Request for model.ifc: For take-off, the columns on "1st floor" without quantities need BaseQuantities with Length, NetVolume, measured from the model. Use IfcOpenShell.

First a look at what the model holds.

```python
import ifcopenshell
import ifcopenshell.util.element
import ifcopenshell.util.unit

model = ifcopenshell.open("model.ifc")
print(model.schema)
for unit_type in ("LENGTHUNIT", "AREAUNIT", "VOLUMEUNIT"):
    print(unit_type, ifcopenshell.util.unit.calculate_unit_scale(model, unit_type))
storey = next(s for s in model.by_type("IfcBuildingStorey") if s.Name == "1st floor")
columns = [e for e in ifcopenshell.util.element.get_decomposition(storey) if e.is_a("IfcColumn")]
for e in sorted(columns, key=lambda e: e.id()):
    print(e.id(), e.is_a(), e.Name, list(ifcopenshell.util.element.get_psets(e, qtos_only=True)), sep=" | ")
```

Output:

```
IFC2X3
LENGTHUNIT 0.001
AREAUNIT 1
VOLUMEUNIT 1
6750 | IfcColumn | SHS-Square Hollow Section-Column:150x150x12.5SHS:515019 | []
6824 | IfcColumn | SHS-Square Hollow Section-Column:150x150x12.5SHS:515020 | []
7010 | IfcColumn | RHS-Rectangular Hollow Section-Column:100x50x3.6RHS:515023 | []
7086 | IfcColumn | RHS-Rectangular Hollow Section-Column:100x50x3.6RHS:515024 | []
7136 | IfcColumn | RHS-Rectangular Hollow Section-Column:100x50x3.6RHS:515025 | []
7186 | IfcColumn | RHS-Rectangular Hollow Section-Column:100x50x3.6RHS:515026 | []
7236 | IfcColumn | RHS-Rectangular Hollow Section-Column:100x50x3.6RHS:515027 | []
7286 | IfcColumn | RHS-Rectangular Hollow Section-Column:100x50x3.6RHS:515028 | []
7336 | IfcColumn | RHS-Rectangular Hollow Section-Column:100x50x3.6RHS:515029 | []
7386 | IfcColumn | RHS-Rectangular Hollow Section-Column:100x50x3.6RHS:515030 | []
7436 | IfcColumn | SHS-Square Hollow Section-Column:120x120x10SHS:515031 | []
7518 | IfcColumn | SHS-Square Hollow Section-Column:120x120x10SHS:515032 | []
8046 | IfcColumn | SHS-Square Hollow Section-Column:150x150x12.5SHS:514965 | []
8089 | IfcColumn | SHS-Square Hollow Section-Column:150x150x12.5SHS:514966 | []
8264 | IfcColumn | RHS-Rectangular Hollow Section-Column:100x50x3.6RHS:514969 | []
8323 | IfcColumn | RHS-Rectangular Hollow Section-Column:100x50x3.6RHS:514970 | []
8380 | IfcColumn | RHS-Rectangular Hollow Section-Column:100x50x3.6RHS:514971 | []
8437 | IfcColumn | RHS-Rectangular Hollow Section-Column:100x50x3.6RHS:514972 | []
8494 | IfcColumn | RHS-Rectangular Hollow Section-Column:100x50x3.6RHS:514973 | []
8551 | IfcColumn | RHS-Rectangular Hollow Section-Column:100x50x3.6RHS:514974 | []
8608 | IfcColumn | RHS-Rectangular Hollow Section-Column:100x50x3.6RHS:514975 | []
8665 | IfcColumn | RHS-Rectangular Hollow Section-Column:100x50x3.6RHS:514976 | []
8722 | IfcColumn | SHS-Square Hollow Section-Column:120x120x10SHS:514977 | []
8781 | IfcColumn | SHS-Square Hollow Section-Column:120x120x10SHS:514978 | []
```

```python
import ifcopenshell
import ifcopenshell.api.pset
import ifcopenshell.geom
import ifcopenshell.util.element
import ifcopenshell.util.shape
import ifcopenshell.util.unit

model = ifcopenshell.open("model.ifc")
unit_scale = ifcopenshell.util.unit.calculate_unit_scale(model)
volume_scale = ifcopenshell.util.unit.calculate_unit_scale(model, "VOLUMEUNIT")
settings = ifcopenshell.geom.settings()

storey = next(s for s in model.by_type("IfcBuildingStorey") if s.Name == "1st floor")
columns = [e for e in ifcopenshell.util.element.get_decomposition(storey) if e.is_a("IfcColumn")]

for e in sorted(columns, key=lambda e: e.id()):
    if ifcopenshell.util.element.get_psets(e, qtos_only=True, should_inherit=False):
        continue
    # Geometry comes back in metres, in the element's own axes.
    shape = ifcopenshell.geom.create_shape(settings, e)
    values = {
        "Length": ifcopenshell.util.shape.get_z(shape.geometry) / unit_scale,
        "NetVolume": ifcopenshell.util.shape.get_volume(shape.geometry) / volume_scale,
    }
    qto = ifcopenshell.api.pset.add_qto(model, product=e, name="BaseQuantities")
    ifcopenshell.api.pset.edit_qto(model, qto=qto, properties=values)
    print(e.id(), {k: round(v, 3) for k, v in values.items()})

model.write("model_edited.ifc")
```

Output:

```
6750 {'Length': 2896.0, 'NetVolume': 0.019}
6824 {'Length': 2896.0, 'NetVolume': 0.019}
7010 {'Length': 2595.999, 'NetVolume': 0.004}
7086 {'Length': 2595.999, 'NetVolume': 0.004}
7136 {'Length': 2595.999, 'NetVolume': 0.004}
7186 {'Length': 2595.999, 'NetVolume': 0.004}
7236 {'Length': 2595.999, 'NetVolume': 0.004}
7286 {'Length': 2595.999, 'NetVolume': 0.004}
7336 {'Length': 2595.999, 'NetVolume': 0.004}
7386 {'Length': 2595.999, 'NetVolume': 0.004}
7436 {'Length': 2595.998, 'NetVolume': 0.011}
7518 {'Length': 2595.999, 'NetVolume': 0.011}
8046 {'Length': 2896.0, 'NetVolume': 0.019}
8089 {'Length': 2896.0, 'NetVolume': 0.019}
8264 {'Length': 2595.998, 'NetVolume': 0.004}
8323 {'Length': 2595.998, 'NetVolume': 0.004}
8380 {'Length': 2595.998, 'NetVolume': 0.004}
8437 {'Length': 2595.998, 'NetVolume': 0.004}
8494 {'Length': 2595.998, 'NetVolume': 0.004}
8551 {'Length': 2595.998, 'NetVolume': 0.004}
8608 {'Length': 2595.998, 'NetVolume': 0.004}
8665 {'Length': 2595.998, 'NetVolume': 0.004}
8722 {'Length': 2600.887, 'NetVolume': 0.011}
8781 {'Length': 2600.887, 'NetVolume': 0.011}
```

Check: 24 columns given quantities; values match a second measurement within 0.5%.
